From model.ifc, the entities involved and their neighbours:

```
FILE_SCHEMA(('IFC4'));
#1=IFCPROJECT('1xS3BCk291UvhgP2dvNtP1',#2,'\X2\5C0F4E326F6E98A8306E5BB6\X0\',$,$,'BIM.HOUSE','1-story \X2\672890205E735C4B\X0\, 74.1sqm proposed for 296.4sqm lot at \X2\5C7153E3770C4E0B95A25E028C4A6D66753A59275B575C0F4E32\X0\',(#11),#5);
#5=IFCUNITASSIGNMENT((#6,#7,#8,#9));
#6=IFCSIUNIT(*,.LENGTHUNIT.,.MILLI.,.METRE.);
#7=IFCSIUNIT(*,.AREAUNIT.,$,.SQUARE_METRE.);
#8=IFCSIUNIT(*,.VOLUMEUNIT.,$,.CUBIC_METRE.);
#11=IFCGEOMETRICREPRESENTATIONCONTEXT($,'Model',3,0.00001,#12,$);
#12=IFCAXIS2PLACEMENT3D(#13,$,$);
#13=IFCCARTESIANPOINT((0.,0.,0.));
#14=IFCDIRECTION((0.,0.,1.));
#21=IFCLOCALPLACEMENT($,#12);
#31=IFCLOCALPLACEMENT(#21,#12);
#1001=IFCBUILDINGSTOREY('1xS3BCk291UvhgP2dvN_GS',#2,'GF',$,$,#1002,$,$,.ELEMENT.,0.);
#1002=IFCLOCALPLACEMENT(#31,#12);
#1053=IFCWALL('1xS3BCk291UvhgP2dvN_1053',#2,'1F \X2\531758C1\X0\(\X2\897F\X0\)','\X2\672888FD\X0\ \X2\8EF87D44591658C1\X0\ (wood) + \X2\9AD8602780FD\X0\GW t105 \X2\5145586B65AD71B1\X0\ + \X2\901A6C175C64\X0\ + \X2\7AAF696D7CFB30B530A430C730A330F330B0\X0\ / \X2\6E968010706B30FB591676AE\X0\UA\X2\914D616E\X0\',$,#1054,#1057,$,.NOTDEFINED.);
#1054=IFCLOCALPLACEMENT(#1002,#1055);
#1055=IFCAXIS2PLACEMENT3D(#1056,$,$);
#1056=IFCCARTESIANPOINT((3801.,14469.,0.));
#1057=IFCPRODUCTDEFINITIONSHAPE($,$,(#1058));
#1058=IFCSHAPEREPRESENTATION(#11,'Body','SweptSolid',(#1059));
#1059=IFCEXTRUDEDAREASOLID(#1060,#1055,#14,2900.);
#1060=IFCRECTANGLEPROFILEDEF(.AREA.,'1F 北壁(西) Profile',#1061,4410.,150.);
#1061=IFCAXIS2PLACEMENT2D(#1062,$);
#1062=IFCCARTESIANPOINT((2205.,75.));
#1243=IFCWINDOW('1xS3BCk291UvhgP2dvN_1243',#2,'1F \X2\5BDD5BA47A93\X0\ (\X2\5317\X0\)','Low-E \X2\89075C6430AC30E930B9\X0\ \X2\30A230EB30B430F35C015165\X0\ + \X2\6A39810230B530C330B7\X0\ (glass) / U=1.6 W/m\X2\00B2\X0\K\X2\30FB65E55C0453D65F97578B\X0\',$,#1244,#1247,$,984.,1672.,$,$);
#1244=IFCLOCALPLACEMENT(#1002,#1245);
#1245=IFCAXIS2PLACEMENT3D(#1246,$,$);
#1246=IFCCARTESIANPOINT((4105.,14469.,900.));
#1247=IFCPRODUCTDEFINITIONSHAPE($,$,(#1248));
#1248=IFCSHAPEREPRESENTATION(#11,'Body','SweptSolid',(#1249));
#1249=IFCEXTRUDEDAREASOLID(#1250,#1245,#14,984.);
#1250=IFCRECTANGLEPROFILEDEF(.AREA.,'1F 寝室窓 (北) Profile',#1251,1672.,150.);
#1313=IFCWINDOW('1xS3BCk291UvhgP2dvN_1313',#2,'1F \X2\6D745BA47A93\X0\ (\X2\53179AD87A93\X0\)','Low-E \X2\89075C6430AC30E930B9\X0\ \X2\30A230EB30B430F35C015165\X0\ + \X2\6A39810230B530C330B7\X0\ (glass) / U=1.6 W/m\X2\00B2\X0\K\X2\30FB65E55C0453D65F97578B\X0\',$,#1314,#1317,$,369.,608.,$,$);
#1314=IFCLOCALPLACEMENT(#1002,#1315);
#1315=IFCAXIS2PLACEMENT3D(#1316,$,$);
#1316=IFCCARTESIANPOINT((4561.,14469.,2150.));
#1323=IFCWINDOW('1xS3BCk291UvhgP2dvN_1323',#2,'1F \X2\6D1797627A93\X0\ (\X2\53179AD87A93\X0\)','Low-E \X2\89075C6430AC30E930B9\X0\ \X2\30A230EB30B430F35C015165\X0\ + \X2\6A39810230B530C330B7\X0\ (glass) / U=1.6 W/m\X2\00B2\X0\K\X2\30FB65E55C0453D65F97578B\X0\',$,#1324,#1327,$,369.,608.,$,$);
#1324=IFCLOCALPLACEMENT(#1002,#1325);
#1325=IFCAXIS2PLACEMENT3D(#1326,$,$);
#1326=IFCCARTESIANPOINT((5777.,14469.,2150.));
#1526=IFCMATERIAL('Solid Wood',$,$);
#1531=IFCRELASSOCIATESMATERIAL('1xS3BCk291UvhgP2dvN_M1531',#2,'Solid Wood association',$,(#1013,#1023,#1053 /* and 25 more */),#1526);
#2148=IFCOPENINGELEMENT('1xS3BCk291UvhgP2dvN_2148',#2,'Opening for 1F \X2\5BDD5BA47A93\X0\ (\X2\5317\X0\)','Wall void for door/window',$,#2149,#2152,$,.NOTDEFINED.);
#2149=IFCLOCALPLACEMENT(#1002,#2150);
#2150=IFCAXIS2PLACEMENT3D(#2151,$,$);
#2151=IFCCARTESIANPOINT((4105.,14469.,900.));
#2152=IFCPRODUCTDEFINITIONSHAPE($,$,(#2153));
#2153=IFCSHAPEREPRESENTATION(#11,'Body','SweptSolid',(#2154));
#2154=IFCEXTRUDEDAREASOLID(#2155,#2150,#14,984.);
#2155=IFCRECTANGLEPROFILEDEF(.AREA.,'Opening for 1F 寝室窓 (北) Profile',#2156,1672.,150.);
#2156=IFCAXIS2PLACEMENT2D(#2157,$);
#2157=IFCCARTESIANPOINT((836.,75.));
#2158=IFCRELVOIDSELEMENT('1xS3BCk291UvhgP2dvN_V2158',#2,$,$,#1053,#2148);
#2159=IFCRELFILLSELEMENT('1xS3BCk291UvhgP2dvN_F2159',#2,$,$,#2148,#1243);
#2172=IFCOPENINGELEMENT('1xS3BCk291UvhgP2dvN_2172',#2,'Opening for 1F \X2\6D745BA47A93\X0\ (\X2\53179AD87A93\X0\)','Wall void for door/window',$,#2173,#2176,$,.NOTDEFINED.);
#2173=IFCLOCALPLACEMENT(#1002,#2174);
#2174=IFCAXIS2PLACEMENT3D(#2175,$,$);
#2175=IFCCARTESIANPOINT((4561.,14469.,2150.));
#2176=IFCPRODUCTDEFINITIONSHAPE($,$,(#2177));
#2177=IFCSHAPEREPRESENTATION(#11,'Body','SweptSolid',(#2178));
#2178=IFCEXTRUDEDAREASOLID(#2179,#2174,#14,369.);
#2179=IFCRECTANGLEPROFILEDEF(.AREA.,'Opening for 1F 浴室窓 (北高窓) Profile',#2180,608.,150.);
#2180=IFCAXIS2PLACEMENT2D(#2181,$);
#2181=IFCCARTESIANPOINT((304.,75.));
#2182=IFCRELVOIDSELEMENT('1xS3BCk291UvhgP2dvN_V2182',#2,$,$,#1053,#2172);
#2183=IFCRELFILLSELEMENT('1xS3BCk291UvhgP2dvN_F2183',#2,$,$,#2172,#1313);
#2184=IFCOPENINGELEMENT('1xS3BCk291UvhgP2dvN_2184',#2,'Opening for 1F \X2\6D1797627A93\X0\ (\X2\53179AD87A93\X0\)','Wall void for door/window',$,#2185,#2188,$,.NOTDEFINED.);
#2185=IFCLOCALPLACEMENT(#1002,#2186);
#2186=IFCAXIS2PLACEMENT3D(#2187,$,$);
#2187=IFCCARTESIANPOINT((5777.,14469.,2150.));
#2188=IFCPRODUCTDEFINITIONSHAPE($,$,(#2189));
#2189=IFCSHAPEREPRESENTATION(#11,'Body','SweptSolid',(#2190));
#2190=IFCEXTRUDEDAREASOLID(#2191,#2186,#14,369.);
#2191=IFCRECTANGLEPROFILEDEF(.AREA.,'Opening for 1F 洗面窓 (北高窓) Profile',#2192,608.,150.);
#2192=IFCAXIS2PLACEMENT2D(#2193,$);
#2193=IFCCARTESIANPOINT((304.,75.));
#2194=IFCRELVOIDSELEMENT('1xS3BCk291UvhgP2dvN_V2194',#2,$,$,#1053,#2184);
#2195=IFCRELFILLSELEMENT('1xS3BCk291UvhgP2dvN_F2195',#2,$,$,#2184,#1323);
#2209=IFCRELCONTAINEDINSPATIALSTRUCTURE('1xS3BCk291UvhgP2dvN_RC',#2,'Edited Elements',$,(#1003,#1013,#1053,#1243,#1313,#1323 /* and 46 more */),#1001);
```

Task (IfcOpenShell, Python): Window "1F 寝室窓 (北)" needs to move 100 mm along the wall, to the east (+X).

```python
import ifcopenshell
import ifcopenshell.api.geometry
import ifcopenshell.util.placement
import ifcopenshell.util.unit

model = ifcopenshell.open("model.ifc")
unit_scale = ifcopenshell.util.unit.calculate_unit_scale(model)

window = model.by_guid("1xS3BCk291UvhgP2dvN_1243")
opening = window.FillsVoids[0].RelatingOpeningElement
wall = opening.VoidsElements[0].RelatingBuildingElement

wall_matrix = ifcopenshell.util.placement.get_local_placement(wall.ObjectPlacement)
shift = wall_matrix[:3, 0] * 0.1 / unit_scale
before = ifcopenshell.util.placement.get_local_placement(window.ObjectPlacement)[:3, 3].copy()

# The window is not placed relative to its opening, so move both.
for product in (opening, window):
    matrix = ifcopenshell.util.placement.get_local_placement(product.ObjectPlacement)
    matrix[:3, 3] += shift
    ifcopenshell.api.geometry.edit_object_placement(model, product=product, matrix=matrix, is_si=False)

after = ifcopenshell.util.placement.get_local_placement(window.ObjectPlacement)[:3, 3]
print("window moved by", (after - before).round(3) + 0.0)

model.write("model_rev.ifc")
```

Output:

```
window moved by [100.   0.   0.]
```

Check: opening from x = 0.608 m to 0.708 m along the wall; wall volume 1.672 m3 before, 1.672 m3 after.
